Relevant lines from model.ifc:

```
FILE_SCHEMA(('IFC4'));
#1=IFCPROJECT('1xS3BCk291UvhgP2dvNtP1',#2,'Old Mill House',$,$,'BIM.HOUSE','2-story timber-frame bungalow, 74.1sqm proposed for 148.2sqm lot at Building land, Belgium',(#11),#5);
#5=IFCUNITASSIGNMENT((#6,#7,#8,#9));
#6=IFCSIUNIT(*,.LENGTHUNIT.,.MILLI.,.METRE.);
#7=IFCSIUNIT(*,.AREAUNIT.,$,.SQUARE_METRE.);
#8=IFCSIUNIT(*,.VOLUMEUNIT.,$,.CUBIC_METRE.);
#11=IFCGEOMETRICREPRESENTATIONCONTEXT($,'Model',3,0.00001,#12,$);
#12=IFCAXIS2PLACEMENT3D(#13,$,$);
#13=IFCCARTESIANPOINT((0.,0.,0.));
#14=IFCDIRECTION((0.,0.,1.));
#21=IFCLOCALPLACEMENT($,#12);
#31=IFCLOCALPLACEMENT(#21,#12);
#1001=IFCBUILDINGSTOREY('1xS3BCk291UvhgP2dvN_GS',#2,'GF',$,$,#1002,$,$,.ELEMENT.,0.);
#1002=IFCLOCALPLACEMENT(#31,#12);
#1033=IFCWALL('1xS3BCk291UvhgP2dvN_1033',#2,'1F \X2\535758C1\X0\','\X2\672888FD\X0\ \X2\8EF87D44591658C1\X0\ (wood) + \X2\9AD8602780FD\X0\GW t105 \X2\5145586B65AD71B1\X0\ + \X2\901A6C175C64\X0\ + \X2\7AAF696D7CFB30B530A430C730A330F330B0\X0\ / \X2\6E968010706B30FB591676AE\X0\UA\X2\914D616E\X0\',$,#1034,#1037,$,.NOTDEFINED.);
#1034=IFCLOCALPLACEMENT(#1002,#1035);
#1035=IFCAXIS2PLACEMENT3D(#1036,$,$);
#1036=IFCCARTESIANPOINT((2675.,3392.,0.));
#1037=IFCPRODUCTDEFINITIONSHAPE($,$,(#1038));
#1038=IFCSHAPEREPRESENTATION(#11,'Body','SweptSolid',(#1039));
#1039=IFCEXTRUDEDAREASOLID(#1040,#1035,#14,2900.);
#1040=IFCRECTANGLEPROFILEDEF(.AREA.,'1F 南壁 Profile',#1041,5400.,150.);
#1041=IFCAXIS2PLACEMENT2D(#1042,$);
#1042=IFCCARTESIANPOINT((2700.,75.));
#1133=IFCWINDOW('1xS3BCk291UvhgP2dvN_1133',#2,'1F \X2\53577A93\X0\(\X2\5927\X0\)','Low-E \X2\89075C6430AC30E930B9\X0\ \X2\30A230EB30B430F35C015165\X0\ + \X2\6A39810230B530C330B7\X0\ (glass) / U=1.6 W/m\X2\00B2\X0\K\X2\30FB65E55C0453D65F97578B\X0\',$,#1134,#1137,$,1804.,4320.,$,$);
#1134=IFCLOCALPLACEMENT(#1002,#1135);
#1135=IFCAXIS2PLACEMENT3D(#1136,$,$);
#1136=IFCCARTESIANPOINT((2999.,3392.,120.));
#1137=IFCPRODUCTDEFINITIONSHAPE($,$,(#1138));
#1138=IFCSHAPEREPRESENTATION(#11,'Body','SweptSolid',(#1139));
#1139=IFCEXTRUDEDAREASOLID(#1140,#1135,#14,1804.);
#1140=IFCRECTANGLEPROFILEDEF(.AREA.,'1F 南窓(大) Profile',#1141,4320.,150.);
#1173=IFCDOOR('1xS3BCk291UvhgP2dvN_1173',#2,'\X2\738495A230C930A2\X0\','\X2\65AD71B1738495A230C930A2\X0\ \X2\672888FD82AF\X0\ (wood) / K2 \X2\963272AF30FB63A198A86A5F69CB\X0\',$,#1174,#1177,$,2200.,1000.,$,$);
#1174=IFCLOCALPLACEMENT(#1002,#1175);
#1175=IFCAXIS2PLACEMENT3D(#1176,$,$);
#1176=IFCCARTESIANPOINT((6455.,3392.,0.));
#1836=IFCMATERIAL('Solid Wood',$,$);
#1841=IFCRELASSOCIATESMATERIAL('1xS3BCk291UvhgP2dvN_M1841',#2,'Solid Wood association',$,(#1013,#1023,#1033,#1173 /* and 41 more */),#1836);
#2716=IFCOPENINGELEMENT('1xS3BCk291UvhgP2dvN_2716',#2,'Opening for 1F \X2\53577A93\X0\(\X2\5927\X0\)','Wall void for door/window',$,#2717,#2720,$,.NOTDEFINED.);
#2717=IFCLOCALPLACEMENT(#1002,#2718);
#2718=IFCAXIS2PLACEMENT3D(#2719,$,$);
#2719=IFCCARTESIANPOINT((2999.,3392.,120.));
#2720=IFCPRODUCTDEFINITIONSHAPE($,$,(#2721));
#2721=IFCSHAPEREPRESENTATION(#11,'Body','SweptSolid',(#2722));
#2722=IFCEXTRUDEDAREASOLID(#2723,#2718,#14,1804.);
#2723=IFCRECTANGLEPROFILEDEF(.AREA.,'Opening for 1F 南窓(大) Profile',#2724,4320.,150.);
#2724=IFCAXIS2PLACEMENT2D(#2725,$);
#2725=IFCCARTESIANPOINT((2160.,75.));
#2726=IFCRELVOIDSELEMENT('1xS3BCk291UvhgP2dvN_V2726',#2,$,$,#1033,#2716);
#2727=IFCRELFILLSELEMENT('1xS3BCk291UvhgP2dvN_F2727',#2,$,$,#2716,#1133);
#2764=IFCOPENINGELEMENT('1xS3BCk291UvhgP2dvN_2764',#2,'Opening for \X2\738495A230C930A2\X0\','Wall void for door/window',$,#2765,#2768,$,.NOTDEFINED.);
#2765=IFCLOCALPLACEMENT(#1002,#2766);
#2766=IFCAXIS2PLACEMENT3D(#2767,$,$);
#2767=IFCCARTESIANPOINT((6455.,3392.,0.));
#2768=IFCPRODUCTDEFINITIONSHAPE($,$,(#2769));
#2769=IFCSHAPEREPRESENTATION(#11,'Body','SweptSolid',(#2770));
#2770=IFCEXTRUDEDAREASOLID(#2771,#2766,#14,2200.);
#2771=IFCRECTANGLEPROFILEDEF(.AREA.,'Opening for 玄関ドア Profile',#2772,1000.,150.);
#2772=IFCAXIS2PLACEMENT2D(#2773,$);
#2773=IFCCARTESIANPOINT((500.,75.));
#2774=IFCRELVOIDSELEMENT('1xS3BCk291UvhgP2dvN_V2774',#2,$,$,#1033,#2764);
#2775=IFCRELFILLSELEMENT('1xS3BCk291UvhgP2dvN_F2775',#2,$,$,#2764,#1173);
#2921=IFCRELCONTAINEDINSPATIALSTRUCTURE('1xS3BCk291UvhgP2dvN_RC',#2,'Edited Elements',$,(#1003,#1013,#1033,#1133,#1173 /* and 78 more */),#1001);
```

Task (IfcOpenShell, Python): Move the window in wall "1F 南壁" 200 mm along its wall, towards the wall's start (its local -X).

```python
import ifcopenshell
import ifcopenshell.api.geometry
import ifcopenshell.util.placement
import ifcopenshell.util.unit

model = ifcopenshell.open("model.ifc")
unit_scale = ifcopenshell.util.unit.calculate_unit_scale(model)

window = model.by_id(1133)
opening = window.FillsVoids[0].RelatingOpeningElement
wall = opening.VoidsElements[0].RelatingBuildingElement

wall_matrix = ifcopenshell.util.placement.get_local_placement(wall.ObjectPlacement)
shift = wall_matrix[:3, 0] * -0.2 / unit_scale
before = ifcopenshell.util.placement.get_local_placement(window.ObjectPlacement)[:3, 3].copy()

# The window is not placed relative to its opening, so move both.
for product in (opening, window):
    matrix = ifcopenshell.util.placement.get_local_placement(product.ObjectPlacement)
    matrix[:3, 3] += shift
    ifcopenshell.api.geometry.edit_object_placement(model, product=product, matrix=matrix, is_si=False)

after = ifcopenshell.util.placement.get_local_placement(window.ObjectPlacement)[:3, 3]
print("window moved by", (after - before).round(3) + 0.0)

model.write("model_v2.ifc")
```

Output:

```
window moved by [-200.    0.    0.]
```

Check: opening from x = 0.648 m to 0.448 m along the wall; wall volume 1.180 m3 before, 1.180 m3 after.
